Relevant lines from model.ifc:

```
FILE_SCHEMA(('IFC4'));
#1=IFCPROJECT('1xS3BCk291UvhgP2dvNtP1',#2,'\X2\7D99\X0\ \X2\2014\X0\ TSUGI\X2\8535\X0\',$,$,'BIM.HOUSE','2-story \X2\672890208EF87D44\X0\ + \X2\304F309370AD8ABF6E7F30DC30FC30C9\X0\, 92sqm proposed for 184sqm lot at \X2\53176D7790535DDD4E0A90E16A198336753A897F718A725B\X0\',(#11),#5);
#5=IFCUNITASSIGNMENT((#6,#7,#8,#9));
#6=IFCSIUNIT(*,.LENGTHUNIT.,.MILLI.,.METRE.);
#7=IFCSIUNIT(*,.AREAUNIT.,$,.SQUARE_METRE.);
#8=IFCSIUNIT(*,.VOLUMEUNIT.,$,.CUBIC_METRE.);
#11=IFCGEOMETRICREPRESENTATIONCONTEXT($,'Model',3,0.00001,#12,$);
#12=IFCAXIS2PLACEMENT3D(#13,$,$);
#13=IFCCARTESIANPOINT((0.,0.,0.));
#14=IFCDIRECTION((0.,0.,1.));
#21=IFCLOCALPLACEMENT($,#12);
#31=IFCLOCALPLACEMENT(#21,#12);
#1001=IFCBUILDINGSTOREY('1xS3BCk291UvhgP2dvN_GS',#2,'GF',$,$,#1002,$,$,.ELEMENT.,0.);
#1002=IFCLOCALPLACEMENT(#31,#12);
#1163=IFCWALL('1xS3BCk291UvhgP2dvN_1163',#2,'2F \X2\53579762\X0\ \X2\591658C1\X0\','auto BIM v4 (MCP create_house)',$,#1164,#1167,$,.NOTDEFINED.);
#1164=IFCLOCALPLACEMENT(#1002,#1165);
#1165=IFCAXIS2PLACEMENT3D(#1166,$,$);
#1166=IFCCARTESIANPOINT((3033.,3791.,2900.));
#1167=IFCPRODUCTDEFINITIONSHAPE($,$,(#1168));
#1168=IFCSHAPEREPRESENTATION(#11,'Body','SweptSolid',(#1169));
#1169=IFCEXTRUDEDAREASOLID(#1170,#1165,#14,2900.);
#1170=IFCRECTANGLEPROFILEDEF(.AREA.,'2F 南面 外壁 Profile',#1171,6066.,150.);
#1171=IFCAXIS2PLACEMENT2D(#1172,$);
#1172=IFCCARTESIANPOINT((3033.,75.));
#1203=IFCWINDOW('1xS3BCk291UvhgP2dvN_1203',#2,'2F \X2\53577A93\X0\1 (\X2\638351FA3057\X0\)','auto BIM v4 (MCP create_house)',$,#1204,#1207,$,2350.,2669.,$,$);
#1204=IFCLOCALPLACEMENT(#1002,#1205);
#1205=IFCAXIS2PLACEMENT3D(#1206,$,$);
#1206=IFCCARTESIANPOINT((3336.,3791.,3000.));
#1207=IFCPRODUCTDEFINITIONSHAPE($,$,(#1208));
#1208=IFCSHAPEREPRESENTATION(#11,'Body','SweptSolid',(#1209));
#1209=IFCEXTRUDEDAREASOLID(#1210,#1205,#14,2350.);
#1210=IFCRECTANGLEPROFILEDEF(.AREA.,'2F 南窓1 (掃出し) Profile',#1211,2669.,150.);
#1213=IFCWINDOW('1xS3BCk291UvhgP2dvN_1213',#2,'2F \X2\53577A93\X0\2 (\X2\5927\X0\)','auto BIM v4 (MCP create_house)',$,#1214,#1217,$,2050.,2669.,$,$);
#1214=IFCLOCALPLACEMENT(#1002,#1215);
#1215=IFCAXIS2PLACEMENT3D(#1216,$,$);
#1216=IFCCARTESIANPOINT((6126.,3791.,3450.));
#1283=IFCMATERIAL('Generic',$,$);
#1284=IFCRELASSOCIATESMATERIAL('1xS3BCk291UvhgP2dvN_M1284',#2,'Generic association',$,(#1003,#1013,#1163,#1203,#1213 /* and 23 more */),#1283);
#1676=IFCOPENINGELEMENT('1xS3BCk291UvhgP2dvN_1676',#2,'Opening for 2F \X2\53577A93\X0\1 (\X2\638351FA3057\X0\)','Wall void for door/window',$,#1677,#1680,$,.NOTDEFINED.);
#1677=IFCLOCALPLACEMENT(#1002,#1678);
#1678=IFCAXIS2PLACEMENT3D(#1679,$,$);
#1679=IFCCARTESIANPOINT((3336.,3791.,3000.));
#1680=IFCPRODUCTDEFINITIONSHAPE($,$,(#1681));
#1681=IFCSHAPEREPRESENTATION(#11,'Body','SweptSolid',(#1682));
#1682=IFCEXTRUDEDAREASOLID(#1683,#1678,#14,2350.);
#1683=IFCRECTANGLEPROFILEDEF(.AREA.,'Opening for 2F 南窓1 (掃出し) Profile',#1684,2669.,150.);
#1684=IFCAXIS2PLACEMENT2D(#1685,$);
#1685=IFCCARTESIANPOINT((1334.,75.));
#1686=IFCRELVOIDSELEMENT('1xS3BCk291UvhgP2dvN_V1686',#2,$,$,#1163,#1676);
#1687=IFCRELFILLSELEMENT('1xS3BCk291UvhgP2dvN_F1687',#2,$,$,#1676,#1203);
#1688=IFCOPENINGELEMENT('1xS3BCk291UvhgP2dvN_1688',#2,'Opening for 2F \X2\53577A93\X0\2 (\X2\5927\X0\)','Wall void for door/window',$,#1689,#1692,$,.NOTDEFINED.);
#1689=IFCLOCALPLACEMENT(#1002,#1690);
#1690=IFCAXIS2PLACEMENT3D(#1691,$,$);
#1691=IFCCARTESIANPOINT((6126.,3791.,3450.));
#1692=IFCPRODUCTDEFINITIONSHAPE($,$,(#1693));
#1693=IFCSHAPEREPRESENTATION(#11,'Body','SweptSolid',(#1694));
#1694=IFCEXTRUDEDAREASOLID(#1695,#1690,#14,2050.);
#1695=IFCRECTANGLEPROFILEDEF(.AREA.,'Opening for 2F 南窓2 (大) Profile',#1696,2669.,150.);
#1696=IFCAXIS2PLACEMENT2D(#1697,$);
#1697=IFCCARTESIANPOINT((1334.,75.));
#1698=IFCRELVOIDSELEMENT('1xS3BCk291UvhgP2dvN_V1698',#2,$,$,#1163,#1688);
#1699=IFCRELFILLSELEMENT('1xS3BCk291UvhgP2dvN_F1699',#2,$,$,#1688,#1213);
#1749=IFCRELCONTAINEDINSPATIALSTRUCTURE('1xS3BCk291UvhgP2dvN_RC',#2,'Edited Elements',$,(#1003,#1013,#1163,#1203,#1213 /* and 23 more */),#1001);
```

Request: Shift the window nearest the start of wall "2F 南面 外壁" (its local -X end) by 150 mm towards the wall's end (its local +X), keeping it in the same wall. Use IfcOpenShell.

```python
import ifcopenshell
import ifcopenshell.api.geometry
import ifcopenshell.util.placement
import ifcopenshell.util.unit

model = ifcopenshell.open("model.ifc")
unit_scale = ifcopenshell.util.unit.calculate_unit_scale(model)

window = model.by_guid("1xS3BCk291UvhgP2dvN_1203")
opening = window.FillsVoids[0].RelatingOpeningElement
wall = opening.VoidsElements[0].RelatingBuildingElement

wall_matrix = ifcopenshell.util.placement.get_local_placement(wall.ObjectPlacement)
shift = wall_matrix[:3, 0] * 0.15 / unit_scale
before = ifcopenshell.util.placement.get_local_placement(window.ObjectPlacement)[:3, 3].copy()

# The window is not placed relative to its opening, so move both.
for product in (opening, window):
    matrix = ifcopenshell.util.placement.get_local_placement(product.ObjectPlacement)
    matrix[:3, 3] += shift
    ifcopenshell.api.geometry.edit_object_placement(model, product=product, matrix=matrix, is_si=False)

after = ifcopenshell.util.placement.get_local_placement(window.ObjectPlacement)[:3, 3]
print("window moved by", (after - before).round(3) + 0.0)

model.write("model_rev.ifc")
```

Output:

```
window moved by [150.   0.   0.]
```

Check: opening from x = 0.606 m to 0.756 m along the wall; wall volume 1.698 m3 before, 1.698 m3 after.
